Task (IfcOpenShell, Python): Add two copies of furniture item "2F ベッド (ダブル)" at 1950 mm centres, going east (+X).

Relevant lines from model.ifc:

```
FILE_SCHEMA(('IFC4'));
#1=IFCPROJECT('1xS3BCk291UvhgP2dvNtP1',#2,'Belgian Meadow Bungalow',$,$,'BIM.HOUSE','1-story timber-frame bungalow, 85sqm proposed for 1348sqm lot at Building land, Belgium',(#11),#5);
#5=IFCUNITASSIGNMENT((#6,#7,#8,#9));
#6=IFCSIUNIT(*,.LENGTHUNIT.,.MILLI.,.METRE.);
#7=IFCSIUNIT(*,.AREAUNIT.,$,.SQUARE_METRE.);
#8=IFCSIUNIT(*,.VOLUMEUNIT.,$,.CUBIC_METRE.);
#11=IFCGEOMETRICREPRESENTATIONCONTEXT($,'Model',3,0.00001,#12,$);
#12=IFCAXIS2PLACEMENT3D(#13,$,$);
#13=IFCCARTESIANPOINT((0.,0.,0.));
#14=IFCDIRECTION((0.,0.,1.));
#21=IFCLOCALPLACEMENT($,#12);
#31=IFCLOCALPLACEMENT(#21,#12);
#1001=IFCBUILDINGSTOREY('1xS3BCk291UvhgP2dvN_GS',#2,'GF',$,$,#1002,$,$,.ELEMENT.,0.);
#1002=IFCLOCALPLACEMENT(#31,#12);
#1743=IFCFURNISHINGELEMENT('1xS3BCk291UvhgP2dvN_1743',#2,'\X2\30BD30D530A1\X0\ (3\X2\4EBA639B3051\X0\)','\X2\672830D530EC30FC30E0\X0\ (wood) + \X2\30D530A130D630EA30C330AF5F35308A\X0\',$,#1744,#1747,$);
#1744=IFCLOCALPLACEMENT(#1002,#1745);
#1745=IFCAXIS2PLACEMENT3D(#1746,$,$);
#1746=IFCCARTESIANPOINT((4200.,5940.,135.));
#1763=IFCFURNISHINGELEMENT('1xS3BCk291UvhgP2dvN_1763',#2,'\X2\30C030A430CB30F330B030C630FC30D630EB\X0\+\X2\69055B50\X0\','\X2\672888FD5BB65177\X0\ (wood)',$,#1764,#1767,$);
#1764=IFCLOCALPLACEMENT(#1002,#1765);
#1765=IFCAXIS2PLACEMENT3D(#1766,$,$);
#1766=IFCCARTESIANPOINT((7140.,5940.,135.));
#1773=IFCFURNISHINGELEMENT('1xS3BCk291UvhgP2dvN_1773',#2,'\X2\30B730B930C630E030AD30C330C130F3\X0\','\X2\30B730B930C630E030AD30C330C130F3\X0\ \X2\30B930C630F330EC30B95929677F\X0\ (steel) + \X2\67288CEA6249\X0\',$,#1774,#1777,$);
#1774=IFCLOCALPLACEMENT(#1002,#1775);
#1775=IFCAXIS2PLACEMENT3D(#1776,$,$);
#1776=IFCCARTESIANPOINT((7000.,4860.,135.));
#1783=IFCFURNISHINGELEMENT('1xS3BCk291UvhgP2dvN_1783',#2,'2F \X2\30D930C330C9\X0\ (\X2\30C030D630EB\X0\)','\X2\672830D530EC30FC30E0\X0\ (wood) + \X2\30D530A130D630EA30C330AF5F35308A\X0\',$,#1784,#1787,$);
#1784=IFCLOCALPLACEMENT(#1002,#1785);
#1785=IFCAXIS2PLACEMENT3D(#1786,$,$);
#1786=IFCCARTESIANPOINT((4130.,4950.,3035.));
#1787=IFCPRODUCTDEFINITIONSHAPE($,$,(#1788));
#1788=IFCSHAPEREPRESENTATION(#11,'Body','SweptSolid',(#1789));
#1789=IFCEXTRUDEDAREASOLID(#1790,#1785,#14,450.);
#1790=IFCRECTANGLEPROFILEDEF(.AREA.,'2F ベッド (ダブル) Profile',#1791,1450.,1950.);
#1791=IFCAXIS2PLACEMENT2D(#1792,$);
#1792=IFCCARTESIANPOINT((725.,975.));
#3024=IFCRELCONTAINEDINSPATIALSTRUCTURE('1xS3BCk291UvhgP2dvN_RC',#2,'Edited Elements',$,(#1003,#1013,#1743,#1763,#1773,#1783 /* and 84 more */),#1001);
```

```python
import numpy as np
import ifcopenshell
import ifcopenshell.api.geometry
import ifcopenshell.api.root
import ifcopenshell.util.element
import ifcopenshell.util.placement

model = ifcopenshell.open("model.ifc")


def reuse_history(source, copy):
    """copy_class also copies each property set's owner history, people and application; keep the originals."""
    for rel in copy.IsDefinedBy:
        if rel.is_a("IfcRelDefinesByProperties") and (history := rel.RelatingPropertyDefinition.OwnerHistory):
            rel.RelatingPropertyDefinition.OwnerHistory = source.OwnerHistory
            ifcopenshell.util.element.remove_deep2(model, history)


source = model.by_guid("1xS3BCk291UvhgP2dvN_1783")
base = ifcopenshell.util.placement.get_local_placement(source.ObjectPlacement)
step = np.array([1.0, 0.0, 0.0]) * 1950.0

for i in range(1, 3):
    copy = ifcopenshell.api.root.copy_class(model, product=source)
    copy.Representation = ifcopenshell.util.element.copy_deep(
        model, source.Representation, exclude=["IfcGeometricRepresentationContext", "IfcRepresentationMap"]
    )
    reuse_history(source, copy)
    matrix = base.copy()
    matrix[:3, 3] += i * step
    print("added at", matrix[:3, 3].round(3) + 0.0)
    ifcopenshell.api.geometry.edit_object_placement(model, product=copy, matrix=matrix, is_si=False)

model.write("model_updated.ifc")
```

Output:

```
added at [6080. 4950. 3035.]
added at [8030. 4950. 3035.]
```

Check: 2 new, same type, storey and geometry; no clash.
